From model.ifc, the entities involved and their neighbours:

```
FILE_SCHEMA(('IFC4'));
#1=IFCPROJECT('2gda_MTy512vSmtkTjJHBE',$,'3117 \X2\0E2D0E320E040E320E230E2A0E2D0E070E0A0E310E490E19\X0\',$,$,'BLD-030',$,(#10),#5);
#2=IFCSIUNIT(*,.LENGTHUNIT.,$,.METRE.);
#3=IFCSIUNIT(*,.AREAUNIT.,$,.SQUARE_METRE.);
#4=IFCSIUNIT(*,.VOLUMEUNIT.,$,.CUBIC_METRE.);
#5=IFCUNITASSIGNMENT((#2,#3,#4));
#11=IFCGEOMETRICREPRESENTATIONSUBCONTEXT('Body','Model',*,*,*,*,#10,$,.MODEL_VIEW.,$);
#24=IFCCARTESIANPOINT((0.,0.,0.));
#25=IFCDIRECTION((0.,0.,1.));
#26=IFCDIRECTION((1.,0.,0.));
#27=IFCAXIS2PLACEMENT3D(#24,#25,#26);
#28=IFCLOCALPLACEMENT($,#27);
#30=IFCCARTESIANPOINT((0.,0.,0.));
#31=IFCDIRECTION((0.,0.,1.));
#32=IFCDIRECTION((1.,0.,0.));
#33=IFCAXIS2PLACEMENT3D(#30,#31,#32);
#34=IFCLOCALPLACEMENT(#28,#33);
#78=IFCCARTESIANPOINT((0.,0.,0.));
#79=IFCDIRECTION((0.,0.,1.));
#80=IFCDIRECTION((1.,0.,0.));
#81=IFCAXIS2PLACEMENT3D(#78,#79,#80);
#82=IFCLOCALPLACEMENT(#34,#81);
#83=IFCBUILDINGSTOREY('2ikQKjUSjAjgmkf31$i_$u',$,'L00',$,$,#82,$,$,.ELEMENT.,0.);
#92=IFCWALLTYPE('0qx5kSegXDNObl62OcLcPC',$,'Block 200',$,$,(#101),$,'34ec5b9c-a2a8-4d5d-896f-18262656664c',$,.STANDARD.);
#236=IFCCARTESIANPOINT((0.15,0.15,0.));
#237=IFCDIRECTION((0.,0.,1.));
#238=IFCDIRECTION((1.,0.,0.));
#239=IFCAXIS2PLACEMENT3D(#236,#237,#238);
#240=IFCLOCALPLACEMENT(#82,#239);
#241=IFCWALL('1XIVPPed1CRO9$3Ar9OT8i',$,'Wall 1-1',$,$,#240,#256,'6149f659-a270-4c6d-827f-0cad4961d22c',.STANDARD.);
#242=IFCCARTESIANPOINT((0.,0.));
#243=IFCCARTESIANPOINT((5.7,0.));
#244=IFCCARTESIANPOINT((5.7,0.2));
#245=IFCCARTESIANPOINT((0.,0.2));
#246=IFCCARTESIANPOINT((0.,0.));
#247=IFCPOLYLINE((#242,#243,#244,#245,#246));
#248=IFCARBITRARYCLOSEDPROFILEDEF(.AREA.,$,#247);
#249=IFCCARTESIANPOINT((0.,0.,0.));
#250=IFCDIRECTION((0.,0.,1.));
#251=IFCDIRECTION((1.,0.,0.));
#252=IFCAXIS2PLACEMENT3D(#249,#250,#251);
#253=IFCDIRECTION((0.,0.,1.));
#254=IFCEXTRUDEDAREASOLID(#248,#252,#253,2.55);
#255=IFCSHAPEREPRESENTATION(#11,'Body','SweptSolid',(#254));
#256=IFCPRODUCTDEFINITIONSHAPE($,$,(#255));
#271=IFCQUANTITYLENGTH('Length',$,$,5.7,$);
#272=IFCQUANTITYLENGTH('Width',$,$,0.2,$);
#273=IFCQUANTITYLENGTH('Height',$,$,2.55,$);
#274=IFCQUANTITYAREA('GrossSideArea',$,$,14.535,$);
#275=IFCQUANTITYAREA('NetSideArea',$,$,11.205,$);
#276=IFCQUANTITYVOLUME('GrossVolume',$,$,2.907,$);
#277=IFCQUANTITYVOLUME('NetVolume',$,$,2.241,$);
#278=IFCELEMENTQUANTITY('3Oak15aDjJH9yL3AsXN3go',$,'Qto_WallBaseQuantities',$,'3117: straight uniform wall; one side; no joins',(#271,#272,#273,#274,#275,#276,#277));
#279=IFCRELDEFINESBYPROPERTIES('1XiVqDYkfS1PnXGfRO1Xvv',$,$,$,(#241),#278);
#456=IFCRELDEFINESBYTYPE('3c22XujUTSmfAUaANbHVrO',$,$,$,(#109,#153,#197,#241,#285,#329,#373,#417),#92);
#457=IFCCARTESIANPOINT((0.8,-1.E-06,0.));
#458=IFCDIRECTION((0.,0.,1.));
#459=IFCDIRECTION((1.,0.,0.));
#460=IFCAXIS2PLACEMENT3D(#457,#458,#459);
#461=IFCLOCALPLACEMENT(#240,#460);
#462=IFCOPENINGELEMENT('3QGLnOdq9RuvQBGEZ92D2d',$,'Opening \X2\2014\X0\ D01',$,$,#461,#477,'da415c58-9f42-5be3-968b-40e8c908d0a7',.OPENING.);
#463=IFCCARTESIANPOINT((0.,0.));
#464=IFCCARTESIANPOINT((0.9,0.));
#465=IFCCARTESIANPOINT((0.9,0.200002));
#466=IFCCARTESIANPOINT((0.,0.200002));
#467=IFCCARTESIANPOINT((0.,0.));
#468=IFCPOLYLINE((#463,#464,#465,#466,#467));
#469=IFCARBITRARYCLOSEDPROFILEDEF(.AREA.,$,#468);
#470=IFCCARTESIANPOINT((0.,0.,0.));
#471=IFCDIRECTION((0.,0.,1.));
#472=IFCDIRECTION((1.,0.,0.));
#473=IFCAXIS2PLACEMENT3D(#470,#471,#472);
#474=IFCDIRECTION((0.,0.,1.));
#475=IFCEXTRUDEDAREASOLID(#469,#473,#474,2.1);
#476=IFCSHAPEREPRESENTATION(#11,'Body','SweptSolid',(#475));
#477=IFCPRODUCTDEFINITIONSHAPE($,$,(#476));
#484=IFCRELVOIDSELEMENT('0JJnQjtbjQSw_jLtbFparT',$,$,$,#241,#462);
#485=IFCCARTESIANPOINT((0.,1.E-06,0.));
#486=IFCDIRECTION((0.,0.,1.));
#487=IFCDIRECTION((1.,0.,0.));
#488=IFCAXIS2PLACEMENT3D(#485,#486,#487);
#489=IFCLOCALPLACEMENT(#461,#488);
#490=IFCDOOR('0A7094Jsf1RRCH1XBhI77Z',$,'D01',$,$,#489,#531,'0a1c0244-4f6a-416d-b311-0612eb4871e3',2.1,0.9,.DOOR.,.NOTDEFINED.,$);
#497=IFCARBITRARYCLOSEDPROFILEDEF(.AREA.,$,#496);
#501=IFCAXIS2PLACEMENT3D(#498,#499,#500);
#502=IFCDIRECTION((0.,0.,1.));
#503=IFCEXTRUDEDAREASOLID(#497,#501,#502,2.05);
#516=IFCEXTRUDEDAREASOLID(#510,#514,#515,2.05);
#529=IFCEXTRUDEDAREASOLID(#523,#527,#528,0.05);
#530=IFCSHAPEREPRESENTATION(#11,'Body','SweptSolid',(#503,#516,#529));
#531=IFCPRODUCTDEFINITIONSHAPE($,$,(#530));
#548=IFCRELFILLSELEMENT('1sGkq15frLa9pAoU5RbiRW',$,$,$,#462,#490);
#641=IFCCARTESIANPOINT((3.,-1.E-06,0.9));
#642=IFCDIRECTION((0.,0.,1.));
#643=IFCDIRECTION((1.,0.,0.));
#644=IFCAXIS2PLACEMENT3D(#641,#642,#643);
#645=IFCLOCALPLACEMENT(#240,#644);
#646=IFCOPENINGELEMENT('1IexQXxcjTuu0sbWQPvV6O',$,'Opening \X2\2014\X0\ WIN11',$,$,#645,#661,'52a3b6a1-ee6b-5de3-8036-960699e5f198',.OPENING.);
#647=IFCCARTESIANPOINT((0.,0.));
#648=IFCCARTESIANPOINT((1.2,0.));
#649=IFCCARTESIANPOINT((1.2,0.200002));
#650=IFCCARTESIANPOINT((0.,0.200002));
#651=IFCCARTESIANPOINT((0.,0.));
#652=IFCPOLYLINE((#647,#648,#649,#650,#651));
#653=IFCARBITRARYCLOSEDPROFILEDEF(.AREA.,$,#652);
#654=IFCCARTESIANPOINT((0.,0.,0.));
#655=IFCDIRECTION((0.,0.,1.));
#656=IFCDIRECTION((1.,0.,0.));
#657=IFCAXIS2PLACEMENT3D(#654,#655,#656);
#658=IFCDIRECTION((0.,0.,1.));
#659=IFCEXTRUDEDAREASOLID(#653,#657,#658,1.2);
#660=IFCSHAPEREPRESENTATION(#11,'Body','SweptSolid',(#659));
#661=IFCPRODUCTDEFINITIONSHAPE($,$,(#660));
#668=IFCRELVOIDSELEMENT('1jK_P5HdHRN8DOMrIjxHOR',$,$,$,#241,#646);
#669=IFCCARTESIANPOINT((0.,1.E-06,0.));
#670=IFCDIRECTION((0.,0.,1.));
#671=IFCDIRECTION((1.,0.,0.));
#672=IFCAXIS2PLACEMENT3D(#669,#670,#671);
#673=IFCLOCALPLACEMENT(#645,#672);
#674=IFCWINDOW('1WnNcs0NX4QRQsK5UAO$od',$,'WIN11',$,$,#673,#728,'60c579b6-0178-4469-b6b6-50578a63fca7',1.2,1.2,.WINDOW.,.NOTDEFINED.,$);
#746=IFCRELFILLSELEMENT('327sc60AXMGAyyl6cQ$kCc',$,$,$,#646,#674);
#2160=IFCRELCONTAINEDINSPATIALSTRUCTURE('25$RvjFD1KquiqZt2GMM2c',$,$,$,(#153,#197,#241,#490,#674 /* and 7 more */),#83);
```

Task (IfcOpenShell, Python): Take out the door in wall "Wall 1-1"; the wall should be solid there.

```python
import ifcopenshell
import ifcopenshell.api.feature
import ifcopenshell.api.pset
import ifcopenshell.api.root
import ifcopenshell.geom
import ifcopenshell.util.element
import ifcopenshell.util.shape
import ifcopenshell.util.unit

model = ifcopenshell.open("model.ifc")
area_scale = ifcopenshell.util.unit.calculate_unit_scale(model, "AREAUNIT")
volume_scale = ifcopenshell.util.unit.calculate_unit_scale(model, "VOLUMEUNIT")
settings = ifcopenshell.geom.settings()


def volume(element):
    """Net volume in cubic metres, openings subtracted."""
    shape = ifcopenshell.geom.create_shape(settings, element)
    return ifcopenshell.util.shape.get_volume(shape.geometry)


door = model.by_guid("0A7094Jsf1RRCH1XBhI77Z")
opening = door.FillsVoids[0].RelatingOpeningElement
wall = opening.VoidsElements[0].RelatingBuildingElement
before = volume(wall)

ifcopenshell.api.root.remove_product(model, product=door)
ifcopenshell.api.feature.remove_feature(model, feature=opening)

after = volume(wall)
thickness = 0.2  # wall thickness in metres

# Update the wall's stored quantities.
qto = model.by_id(ifcopenshell.util.element.get_pset(wall, "Qto_WallBaseQuantities", should_inherit=False)["id"])
ifcopenshell.api.pset.edit_qto(model, qto=qto, properties={
    "NetSideArea": after / thickness / area_scale,
    "NetVolume": after / volume_scale,
})

print(f"wall volume {before:.3f} -> {after:.3f} m3")

model.write("model_v2.ifc")
```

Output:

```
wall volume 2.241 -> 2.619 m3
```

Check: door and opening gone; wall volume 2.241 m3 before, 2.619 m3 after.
